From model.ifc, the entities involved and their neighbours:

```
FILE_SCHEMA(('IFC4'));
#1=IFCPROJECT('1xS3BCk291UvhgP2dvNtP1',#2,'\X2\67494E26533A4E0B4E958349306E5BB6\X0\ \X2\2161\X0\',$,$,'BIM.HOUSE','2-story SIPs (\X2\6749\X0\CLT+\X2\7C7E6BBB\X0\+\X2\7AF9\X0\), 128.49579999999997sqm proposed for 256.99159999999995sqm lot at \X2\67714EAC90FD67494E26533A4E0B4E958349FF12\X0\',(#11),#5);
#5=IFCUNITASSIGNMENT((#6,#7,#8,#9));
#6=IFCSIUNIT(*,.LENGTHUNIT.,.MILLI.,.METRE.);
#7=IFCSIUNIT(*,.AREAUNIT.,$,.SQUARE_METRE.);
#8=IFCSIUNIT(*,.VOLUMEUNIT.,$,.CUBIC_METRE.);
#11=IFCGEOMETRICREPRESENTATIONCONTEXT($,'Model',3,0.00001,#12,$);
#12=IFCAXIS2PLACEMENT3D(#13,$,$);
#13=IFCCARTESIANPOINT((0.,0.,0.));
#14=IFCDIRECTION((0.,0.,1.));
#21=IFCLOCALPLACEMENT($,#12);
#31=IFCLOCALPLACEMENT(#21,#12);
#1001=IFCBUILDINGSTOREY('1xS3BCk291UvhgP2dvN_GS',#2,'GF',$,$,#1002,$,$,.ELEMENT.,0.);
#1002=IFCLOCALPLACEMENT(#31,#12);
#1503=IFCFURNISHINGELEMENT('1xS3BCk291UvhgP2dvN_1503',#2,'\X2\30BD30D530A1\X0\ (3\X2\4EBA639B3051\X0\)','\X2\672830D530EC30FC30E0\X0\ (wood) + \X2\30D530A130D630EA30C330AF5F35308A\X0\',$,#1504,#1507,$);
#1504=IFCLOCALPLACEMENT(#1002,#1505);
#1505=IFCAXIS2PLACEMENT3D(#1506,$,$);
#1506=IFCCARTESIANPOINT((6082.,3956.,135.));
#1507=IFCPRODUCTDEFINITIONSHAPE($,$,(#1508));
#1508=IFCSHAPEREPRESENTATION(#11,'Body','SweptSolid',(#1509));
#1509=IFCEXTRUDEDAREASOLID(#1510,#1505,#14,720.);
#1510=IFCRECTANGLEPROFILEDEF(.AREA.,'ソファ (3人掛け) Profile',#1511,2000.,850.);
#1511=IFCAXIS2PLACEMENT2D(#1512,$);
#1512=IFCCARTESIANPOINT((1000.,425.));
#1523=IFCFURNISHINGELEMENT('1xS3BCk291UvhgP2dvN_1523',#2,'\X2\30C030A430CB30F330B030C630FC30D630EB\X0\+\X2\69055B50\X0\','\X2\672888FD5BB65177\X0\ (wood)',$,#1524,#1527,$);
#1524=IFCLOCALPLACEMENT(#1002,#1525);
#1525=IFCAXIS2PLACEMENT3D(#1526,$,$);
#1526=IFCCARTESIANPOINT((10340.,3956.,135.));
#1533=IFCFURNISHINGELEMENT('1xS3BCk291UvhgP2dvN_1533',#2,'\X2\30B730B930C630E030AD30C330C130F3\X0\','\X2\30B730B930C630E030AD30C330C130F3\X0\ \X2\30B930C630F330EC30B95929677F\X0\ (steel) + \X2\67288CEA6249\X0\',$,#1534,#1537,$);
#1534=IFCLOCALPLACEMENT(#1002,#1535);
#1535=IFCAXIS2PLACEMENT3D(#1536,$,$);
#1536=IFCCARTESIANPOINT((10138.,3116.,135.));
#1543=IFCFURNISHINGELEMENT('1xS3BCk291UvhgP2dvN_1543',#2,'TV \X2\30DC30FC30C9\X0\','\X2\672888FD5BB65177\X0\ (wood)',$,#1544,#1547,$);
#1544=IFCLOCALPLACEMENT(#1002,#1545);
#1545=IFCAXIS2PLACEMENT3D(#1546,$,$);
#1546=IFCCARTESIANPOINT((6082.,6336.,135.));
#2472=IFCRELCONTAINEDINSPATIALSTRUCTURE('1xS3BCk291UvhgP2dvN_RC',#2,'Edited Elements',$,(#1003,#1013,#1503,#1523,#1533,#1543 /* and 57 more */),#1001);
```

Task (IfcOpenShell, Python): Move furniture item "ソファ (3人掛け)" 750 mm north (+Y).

```python
import ifcopenshell
import ifcopenshell.api.geometry
import ifcopenshell.util.placement
import ifcopenshell.util.unit

model = ifcopenshell.open("model.ifc")
unit_scale = ifcopenshell.util.unit.calculate_unit_scale(model)

item = model.by_guid("1xS3BCk291UvhgP2dvN_1503")
matrix = ifcopenshell.util.placement.get_local_placement(item.ObjectPlacement)
matrix[1, 3] += 0.75 / unit_scale
ifcopenshell.api.geometry.edit_object_placement(model, product=item, matrix=matrix, is_si=False)

print(ifcopenshell.util.placement.get_local_placement(item.ObjectPlacement).round(3) + 0.0)

model.write("model_v2.ifc")
```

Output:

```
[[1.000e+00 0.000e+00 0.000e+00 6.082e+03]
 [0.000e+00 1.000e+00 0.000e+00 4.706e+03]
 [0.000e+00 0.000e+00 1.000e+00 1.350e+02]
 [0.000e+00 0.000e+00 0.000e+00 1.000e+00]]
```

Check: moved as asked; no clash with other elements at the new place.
